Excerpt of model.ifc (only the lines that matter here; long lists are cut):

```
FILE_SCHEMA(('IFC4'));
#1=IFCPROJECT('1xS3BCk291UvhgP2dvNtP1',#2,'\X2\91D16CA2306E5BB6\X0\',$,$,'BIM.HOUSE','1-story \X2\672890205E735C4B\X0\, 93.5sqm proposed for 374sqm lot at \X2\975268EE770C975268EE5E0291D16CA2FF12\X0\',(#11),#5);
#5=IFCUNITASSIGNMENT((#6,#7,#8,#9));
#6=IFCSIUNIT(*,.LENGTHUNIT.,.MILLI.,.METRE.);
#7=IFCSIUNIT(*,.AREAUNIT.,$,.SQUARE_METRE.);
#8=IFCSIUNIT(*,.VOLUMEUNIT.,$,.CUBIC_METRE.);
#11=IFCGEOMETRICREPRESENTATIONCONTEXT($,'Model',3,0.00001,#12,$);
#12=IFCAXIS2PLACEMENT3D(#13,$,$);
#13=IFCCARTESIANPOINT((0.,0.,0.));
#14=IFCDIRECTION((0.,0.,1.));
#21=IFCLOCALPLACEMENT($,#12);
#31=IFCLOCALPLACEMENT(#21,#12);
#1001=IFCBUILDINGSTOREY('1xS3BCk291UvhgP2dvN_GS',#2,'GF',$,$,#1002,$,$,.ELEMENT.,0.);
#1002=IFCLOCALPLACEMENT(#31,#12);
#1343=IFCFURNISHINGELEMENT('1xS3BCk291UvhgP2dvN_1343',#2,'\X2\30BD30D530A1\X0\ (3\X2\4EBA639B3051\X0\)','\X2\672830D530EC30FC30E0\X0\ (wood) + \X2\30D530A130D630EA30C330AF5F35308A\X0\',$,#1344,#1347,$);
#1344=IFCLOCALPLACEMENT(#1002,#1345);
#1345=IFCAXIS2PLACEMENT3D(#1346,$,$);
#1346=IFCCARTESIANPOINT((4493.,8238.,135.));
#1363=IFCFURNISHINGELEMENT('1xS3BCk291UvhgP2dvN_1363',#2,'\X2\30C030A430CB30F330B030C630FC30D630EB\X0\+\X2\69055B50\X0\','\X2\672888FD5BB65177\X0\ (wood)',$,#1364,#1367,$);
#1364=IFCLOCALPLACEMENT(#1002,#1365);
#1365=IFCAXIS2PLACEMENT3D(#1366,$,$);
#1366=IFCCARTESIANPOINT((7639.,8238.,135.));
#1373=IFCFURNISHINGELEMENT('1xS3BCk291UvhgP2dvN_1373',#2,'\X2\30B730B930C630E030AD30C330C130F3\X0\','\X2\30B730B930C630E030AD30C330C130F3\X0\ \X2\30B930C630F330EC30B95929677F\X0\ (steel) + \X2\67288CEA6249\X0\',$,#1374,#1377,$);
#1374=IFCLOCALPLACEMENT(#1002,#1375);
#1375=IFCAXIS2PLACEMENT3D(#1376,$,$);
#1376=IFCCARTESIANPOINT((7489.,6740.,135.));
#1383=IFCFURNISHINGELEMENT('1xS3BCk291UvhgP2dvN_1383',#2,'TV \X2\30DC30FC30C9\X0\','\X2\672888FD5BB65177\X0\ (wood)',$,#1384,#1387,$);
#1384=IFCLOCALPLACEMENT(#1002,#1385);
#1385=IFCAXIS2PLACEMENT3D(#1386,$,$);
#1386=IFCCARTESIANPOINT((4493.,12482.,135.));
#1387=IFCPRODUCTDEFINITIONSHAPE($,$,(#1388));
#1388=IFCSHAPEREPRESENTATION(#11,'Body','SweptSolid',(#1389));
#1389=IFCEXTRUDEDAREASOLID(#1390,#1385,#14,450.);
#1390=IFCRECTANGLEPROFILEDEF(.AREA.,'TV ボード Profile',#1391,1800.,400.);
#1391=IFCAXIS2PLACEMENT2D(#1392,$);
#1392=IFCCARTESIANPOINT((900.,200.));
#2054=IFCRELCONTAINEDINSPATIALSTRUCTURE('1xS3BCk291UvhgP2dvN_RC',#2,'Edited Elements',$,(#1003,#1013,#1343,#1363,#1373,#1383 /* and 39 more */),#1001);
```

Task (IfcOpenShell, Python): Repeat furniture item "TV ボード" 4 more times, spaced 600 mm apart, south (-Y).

```python
import numpy as np
import ifcopenshell
import ifcopenshell.api.geometry
import ifcopenshell.api.root
import ifcopenshell.util.element
import ifcopenshell.util.placement
import ifcopenshell.util.unit

model = ifcopenshell.open("model.ifc")
unit_scale = ifcopenshell.util.unit.calculate_unit_scale(model)


def reuse_history(source, copy):
    """copy_class also copies each property set's owner history, people and application; keep the originals."""
    for rel in copy.IsDefinedBy:
        if rel.is_a("IfcRelDefinesByProperties") and (history := rel.RelatingPropertyDefinition.OwnerHistory):
            rel.RelatingPropertyDefinition.OwnerHistory = source.OwnerHistory
            ifcopenshell.util.element.remove_deep2(model, history)


source = model.by_id(1383)
base = ifcopenshell.util.placement.get_local_placement(source.ObjectPlacement)
step = np.array([0.0, -1.0, 0.0]) * 0.6 / unit_scale

for i in range(1, 5):
    copy = ifcopenshell.api.root.copy_class(model, product=source)
    copy.Representation = ifcopenshell.util.element.copy_deep(
        model, source.Representation, exclude=["IfcGeometricRepresentationContext", "IfcRepresentationMap"]
    )
    reuse_history(source, copy)
    matrix = base.copy()
    matrix[:3, 3] += i * step
    print("added at", matrix[:3, 3].round(3) + 0.0)
    ifcopenshell.api.geometry.edit_object_placement(model, product=copy, matrix=matrix, is_si=False)

model.write("model_edited.ifc")
```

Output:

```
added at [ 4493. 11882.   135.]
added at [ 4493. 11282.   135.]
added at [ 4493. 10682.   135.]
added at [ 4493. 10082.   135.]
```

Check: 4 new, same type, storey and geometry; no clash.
